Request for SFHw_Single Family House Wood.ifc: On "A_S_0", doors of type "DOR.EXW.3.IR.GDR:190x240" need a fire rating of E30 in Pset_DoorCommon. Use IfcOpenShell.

First a look at what the model holds.

```python
import ifcopenshell
import ifcopenshell.util.element

model = ifcopenshell.open("SFHw_Single Family House Wood.ifc")
print(model.schema)
storey = next(s for s in model.by_type("IfcBuildingStorey") if s.Name == "A_S_0")
doors = [e for e in ifcopenshell.util.element.get_decomposition(storey) if e.is_a("IfcDoor")]
seen = {}
for e in doors:
    element_type = ifcopenshell.util.element.get_type(e)
    key = (element_type.Name if element_type != e and element_type else None, ifcopenshell.util.element.get_pset(e, "Pset_DoorCommon", "FireRating"))
    seen[key] = seen.get(key, 0) + 1
for (name, value), count in sorted(seen.items(), key=str):
    print(count, "x", name, "|", value)
```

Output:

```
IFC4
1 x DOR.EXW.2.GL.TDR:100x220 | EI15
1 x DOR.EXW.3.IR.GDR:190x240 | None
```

```python
import ifcopenshell
import ifcopenshell.api.pset
import ifcopenshell.util.element

model = ifcopenshell.open("SFHw_Single Family House Wood.ifc")

storey = next(s for s in model.by_type("IfcBuildingStorey") if s.Name == "A_S_0")
doors = [e for e in ifcopenshell.util.element.get_decomposition(storey) if e.is_a("IfcDoor")]

count = 0
for e in doors:
    element_type = ifcopenshell.util.element.get_type(e)
    if element_type in (None, e) or element_type.Name != "DOR.EXW.3.IR.GDR:190x240":
        continue
    # add_pset returns the element's existing set when there is one.
    pset = ifcopenshell.api.pset.add_pset(model, product=e, name="Pset_DoorCommon")
    ifcopenshell.api.pset.edit_pset(model, pset=pset, properties={"FireRating": "E30"})
    count += 1

print(count, "doors updated")

model.write("SFHw_Single Family House Wood_updated.ifc")
```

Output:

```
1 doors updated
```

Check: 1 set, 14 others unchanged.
